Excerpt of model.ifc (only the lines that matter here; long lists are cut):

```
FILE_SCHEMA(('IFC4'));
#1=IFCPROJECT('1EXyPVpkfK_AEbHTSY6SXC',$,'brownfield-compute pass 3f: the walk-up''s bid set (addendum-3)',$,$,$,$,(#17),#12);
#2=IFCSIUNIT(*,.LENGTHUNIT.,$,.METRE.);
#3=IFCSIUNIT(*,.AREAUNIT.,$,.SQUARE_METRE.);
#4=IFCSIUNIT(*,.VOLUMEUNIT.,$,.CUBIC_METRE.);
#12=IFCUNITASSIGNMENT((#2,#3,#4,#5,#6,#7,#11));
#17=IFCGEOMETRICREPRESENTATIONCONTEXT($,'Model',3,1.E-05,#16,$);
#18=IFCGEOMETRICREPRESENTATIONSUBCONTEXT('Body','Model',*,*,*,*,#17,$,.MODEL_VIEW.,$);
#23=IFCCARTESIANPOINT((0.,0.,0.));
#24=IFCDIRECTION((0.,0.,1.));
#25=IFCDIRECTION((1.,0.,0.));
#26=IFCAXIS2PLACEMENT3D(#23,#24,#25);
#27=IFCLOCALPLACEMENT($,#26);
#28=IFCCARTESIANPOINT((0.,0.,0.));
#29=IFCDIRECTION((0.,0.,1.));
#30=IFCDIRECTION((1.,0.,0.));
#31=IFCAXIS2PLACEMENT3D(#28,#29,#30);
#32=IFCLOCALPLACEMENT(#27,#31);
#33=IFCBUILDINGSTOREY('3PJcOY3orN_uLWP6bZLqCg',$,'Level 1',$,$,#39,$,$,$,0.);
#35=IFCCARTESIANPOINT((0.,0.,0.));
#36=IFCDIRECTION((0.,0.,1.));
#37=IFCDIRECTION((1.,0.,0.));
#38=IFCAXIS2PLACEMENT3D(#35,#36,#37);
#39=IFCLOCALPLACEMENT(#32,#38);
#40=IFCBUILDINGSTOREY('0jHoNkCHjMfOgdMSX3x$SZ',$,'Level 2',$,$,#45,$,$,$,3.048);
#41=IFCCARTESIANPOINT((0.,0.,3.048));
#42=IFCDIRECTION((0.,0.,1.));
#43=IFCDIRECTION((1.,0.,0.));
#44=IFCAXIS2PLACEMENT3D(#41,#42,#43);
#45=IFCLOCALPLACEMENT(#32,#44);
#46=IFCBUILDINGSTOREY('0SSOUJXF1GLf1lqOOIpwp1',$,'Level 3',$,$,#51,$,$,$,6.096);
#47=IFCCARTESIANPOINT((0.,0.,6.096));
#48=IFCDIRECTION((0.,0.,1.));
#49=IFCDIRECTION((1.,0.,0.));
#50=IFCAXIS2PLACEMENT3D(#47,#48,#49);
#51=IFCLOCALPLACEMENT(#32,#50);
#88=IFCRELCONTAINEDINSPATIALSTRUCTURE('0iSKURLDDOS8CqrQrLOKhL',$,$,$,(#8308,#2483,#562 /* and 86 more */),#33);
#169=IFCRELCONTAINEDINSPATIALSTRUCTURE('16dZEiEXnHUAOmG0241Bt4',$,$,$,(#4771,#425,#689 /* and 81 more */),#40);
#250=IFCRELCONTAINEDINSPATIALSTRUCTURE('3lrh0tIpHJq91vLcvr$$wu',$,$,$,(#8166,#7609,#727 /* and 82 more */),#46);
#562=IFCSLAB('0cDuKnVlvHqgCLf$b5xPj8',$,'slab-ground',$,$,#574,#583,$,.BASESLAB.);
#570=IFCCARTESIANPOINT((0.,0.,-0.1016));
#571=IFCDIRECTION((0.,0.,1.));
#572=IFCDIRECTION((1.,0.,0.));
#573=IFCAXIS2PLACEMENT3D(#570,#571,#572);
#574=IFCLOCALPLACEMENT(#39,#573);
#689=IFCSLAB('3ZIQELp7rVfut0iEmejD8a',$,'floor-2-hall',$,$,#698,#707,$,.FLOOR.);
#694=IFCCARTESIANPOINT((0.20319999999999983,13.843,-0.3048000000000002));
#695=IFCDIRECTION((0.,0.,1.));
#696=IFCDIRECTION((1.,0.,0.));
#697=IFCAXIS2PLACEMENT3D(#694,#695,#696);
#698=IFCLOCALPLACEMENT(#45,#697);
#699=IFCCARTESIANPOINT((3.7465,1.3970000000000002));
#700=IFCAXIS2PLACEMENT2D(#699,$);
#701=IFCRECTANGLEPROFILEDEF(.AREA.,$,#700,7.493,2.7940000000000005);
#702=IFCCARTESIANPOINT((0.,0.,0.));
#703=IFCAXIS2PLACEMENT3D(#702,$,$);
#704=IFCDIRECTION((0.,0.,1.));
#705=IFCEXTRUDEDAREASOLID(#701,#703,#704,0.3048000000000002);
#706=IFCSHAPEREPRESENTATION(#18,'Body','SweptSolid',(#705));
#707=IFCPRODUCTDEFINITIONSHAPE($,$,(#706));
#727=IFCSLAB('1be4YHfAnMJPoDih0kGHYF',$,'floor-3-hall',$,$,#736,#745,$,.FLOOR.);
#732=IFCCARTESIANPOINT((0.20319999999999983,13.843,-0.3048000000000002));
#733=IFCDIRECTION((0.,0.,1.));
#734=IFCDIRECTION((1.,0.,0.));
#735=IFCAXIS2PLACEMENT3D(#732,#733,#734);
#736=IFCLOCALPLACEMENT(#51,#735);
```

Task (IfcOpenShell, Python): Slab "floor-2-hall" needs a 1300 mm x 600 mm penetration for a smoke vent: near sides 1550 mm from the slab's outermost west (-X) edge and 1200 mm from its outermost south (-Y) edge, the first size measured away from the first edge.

```python
import numpy as np
import ifcopenshell
import ifcopenshell.api.feature
import ifcopenshell.api.geometry
import ifcopenshell.api.root
import ifcopenshell.geom
import ifcopenshell.util.placement
import ifcopenshell.util.representation
import ifcopenshell.util.shape
import ifcopenshell.util.unit

model = ifcopenshell.open("model.ifc")
unit_scale = ifcopenshell.util.unit.calculate_unit_scale(model)
settings = ifcopenshell.geom.settings()


def volume(element):
    """Net volume in cubic metres, openings subtracted."""
    shape = ifcopenshell.geom.create_shape(settings, element)
    return ifcopenshell.util.shape.get_volume(shape.geometry)


slab = model.by_guid("3ZIQELp7rVfut0iEmejD8a")
before = volume(slab)

# Extent in the slab's own axes, in metres. The edges named are its -X and -Y sides.
slab_shape = ifcopenshell.geom.create_shape(settings, slab)
vertices = ifcopenshell.util.shape.get_vertices(slab_shape.geometry)
x_min, y_min, bottom = vertices.min(axis=0)
top = vertices[:, 2].max()

opening = ifcopenshell.api.root.create_entity(model, ifc_class="IfcOpeningElement", name="Smoke vent opening", predefined_type="OPENING")
context = ifcopenshell.util.representation.get_context(model, "Model", "Body", "MODEL_VIEW")
width, depth = 1.3, 0.6
outline = [(0.0, 0.0), (width, 0.0), (width, depth), (0.0, depth), (0.0, 0.0)]
# Overshoot both faces by 50 mm so the cut is clean.
shape = ifcopenshell.api.geometry.add_slab_representation(
    model, context=context, depth=top - bottom + 0.1, polyline=outline
)
ifcopenshell.api.geometry.assign_representation(model, product=opening, representation=shape)

matrix = ifcopenshell.util.placement.get_local_placement(slab.ObjectPlacement)
matrix[:, 3] = matrix @ np.append(np.array([x_min + 1.55, y_min + 1.2, bottom - 0.05]) / unit_scale, 1.0)
ifcopenshell.api.geometry.edit_object_placement(model, product=opening, matrix=matrix, is_si=False)
ifcopenshell.api.feature.add_feature(model, feature=opening, element=slab)

after = volume(slab)

print(f"slab volume {before:.3f} -> {after:.3f} m3")

model.write("model_updated.ifc")
```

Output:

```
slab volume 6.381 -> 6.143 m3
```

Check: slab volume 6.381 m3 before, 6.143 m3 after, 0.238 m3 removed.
